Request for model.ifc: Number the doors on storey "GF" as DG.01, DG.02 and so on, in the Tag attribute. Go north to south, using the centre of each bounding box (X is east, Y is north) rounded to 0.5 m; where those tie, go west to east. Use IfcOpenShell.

First a look at what the model holds.

```python
import ifcopenshell
import ifcopenshell.util.element
import ifcopenshell.util.placement

model = ifcopenshell.open("model.ifc")
print(model.schema)
storey = next(s for s in model.by_type("IfcBuildingStorey") if s.Name == "GF")
doors = [e for e in ifcopenshell.util.element.get_decomposition(storey) if e.is_a("IfcDoor")]
for e in sorted(doors, key=lambda e: e.id()):
    origin = ifcopenshell.util.placement.get_local_placement(e.ObjectPlacement)[:3, 3]
    print(e.id(), e.Tag, e.Name, origin.round(2) + 0.0, sep=" | ")
```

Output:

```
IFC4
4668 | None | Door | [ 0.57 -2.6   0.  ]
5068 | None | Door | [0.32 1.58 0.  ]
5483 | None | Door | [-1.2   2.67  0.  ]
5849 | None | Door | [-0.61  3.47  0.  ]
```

```python
import ifcopenshell
import ifcopenshell.geom
import ifcopenshell.util.element
import ifcopenshell.util.shape

model = ifcopenshell.open("model.ifc")
settings = ifcopenshell.geom.settings()
settings.set("use-world-coords", True)


def centre(element):
    shape = ifcopenshell.geom.create_shape(settings, element)
    return ifcopenshell.util.shape.get_bbox_centroid(shape.geometry)


storey = next(s for s in model.by_type("IfcBuildingStorey") if s.Name == "GF")
doors = [e for e in ifcopenshell.util.element.get_decomposition(storey) if e.is_a("IfcDoor")]

# Insertion points can sit at a corner or the storey origin, so sort by the geometry (in metres).
centres = {e: centre(e) for e in doors}
doors.sort(key=lambda e: (-round(centres[e][1] / 0.5), centres[e][0]))

for i, e in enumerate(doors, start=1):
    number = f"DG.{i:02d}"
    e.Tag = number
    print(e.id(), number)

model.write("model_v2.ifc")
```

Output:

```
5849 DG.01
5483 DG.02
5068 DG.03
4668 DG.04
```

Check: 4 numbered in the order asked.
